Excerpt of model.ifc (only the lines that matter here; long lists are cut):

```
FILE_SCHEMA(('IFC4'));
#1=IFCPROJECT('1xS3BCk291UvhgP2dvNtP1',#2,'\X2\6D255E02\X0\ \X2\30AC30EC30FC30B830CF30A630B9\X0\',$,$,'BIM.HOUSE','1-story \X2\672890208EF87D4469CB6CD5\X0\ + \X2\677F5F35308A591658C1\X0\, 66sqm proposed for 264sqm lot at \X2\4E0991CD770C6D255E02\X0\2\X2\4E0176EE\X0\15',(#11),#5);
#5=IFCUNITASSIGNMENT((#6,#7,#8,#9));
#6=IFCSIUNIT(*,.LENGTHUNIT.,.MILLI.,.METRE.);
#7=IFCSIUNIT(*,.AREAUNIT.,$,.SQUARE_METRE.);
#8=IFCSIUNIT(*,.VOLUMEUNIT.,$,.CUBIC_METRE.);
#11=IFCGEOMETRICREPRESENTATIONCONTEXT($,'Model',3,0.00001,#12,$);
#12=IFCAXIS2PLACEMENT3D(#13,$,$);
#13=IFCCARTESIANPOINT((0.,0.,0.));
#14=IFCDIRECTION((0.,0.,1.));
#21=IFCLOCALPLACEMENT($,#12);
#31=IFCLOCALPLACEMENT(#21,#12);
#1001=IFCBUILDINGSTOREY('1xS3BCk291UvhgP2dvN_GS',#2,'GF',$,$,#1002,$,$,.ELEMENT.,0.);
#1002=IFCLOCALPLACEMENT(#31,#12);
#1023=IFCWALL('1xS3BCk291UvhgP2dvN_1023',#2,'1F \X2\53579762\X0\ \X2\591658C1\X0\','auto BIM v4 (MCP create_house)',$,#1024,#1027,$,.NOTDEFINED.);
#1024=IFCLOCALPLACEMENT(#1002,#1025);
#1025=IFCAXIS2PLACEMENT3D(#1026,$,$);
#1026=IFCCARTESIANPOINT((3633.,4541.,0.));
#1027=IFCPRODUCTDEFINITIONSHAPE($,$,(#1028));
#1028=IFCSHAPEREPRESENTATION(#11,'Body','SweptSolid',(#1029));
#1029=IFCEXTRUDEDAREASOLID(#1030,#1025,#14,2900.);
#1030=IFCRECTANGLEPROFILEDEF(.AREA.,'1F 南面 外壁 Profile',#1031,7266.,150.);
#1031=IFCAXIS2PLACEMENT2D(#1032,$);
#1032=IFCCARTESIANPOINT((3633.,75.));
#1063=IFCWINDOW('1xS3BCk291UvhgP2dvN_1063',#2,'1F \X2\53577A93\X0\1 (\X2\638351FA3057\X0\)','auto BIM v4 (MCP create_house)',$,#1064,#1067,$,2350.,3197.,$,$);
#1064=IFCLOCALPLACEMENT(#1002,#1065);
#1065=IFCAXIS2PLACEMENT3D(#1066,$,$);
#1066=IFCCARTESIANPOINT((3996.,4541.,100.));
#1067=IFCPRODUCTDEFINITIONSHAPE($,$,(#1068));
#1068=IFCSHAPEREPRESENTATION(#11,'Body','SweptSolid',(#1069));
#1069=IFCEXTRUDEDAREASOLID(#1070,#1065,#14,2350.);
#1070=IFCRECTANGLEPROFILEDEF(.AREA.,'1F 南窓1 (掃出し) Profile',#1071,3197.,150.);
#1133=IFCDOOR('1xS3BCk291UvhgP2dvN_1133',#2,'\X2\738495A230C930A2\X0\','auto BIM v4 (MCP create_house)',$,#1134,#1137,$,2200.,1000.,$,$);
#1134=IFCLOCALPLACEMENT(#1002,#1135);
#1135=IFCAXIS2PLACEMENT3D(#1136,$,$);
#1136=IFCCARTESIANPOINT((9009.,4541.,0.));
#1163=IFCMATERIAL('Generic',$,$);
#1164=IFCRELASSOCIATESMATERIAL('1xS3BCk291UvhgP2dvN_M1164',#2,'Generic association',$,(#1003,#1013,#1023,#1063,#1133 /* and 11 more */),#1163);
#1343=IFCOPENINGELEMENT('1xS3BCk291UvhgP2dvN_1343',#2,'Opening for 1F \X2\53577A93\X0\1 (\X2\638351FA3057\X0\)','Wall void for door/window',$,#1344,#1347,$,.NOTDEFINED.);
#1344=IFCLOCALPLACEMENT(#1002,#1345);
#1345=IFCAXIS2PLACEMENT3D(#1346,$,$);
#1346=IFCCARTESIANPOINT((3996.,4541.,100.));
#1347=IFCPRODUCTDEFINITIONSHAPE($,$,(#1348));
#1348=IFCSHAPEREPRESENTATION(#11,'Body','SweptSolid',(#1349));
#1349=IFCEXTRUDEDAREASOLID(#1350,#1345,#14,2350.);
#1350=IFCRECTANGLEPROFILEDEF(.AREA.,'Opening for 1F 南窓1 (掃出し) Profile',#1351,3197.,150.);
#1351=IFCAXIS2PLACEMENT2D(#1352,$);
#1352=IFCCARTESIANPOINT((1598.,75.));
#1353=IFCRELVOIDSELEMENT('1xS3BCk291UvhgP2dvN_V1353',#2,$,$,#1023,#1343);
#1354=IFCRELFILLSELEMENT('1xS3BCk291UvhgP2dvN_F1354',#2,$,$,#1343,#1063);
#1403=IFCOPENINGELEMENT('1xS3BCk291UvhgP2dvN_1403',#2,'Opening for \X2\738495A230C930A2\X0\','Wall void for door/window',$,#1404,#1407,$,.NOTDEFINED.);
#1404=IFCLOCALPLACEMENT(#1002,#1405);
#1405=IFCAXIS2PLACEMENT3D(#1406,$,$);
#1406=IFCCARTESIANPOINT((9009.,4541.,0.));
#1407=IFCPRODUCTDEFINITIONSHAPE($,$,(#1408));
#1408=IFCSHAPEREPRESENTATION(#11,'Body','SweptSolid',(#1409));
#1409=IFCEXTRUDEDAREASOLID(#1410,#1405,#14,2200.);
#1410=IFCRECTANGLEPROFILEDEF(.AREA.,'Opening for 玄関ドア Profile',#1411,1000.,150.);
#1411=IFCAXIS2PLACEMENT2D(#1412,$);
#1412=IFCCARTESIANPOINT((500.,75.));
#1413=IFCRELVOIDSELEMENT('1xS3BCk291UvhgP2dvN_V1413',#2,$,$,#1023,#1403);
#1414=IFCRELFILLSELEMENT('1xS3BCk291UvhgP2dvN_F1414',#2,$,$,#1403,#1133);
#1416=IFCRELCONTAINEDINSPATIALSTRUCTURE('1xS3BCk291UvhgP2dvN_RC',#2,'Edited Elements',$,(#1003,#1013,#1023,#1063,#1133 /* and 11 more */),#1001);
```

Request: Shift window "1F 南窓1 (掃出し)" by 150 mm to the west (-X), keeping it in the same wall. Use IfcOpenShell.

```python
import ifcopenshell
import ifcopenshell.api.geometry
import ifcopenshell.util.placement
import ifcopenshell.util.unit

model = ifcopenshell.open("model.ifc")
unit_scale = ifcopenshell.util.unit.calculate_unit_scale(model)

window = model.by_guid("1xS3BCk291UvhgP2dvN_1063")
opening = window.FillsVoids[0].RelatingOpeningElement
wall = opening.VoidsElements[0].RelatingBuildingElement

wall_matrix = ifcopenshell.util.placement.get_local_placement(wall.ObjectPlacement)
shift = wall_matrix[:3, 0] * -0.15 / unit_scale
before = ifcopenshell.util.placement.get_local_placement(window.ObjectPlacement)[:3, 3].copy()

# The window is not placed relative to its opening, so move both.
for product in (opening, window):
    matrix = ifcopenshell.util.placement.get_local_placement(product.ObjectPlacement)
    matrix[:3, 3] += shift
    ifcopenshell.api.geometry.edit_object_placement(model, product=product, matrix=matrix, is_si=False)

after = ifcopenshell.util.placement.get_local_placement(window.ObjectPlacement)[:3, 3]
print("window moved by", (after - before).round(3) + 0.0)

model.write("model_rev.ifc")
```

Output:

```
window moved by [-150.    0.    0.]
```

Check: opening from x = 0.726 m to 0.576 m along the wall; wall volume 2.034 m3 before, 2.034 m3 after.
